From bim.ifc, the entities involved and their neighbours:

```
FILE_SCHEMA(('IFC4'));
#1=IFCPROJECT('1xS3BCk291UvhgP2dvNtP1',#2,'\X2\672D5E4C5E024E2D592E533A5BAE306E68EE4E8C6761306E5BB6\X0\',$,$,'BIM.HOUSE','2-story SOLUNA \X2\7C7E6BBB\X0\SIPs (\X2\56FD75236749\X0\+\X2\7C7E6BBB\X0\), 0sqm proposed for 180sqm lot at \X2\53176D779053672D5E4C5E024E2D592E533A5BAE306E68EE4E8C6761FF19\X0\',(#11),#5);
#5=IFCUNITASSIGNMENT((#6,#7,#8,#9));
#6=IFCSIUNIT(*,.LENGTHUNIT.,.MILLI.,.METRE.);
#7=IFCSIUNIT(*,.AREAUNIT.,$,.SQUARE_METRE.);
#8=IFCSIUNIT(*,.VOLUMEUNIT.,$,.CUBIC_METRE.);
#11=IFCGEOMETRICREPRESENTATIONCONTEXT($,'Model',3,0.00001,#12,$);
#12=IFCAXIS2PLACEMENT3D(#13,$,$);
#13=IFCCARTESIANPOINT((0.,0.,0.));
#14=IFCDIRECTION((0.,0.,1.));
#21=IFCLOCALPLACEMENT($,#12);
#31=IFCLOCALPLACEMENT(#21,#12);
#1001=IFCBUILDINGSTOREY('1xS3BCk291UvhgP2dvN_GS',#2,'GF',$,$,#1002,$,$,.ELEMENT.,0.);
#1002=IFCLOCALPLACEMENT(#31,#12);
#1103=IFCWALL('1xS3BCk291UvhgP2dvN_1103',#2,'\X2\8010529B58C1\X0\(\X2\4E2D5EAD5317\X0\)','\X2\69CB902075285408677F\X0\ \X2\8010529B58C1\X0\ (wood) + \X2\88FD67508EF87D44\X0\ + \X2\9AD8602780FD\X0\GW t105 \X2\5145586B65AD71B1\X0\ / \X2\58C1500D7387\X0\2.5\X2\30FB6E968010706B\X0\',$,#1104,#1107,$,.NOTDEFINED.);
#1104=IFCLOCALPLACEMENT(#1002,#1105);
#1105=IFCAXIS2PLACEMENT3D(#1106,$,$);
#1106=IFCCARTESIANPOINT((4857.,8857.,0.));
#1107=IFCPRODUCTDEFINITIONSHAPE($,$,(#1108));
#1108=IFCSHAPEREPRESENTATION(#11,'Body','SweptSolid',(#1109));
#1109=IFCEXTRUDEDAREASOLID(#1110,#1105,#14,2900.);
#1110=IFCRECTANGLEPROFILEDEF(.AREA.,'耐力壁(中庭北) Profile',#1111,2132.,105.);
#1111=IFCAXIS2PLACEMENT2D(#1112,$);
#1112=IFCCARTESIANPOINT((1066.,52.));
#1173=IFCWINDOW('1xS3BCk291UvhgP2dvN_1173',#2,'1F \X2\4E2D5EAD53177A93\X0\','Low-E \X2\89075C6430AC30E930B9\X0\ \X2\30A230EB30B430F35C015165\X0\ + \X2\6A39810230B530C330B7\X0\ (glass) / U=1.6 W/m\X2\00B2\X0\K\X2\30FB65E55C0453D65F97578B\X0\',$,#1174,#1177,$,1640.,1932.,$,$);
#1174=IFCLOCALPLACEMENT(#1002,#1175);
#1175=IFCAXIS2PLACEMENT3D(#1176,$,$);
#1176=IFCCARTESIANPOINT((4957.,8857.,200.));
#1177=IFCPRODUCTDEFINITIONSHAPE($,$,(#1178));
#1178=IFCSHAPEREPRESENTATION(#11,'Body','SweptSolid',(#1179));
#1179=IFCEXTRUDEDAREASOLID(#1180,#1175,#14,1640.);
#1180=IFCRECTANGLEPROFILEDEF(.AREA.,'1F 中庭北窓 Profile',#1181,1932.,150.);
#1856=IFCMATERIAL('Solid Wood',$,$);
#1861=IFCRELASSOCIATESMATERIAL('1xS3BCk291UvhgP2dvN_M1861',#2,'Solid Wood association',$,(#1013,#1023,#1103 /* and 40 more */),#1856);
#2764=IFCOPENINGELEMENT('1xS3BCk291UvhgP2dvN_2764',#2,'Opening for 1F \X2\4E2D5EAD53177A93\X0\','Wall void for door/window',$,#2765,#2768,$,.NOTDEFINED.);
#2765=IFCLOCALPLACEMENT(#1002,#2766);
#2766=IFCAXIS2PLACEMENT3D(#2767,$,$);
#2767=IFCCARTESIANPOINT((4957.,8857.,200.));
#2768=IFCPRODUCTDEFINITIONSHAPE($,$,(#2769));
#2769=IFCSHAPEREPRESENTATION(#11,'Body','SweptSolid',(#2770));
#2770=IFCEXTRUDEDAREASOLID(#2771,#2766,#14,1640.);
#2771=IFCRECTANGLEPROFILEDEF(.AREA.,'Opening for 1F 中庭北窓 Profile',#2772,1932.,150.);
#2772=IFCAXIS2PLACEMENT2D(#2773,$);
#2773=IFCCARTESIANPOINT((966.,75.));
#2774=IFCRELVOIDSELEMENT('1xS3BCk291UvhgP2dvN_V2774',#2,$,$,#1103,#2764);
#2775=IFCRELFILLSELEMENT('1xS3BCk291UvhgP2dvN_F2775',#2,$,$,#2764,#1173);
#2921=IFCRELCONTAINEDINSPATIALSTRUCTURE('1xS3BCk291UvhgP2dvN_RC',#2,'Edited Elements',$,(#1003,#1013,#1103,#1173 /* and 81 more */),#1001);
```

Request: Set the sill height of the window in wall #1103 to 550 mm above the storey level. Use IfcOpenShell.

```python
import numpy as np
import ifcopenshell
import ifcopenshell.api.geometry
import ifcopenshell.geom
import ifcopenshell.util.element
import ifcopenshell.util.placement
import ifcopenshell.util.shape
import ifcopenshell.util.unit

model = ifcopenshell.open("bim.ifc")
unit_scale = ifcopenshell.util.unit.calculate_unit_scale(model)

window = model.by_id(1173)
opening = window.FillsVoids[0].RelatingOpeningElement
storey = ifcopenshell.util.element.get_container(window, ifc_class="IfcBuildingStorey")
level = ifcopenshell.util.placement.get_local_placement(storey.ObjectPlacement)[2, 3]

# The opening's origin need not be at the sill, so measure its lowest point.
shape = ifcopenshell.geom.create_shape(ifcopenshell.geom.settings(), opening)
bottom = ifcopenshell.util.shape.get_shape_bottom_elevation(shape, shape.geometry) / unit_scale
dz = level + 550.0 - bottom

shift = np.array([0.0, 0.0, dz])
# The window is not placed relative to its opening, so move both.
for product in (opening, window):
    matrix = ifcopenshell.util.placement.get_local_placement(product.ObjectPlacement)
    matrix[:3, 3] += shift
    ifcopenshell.api.geometry.edit_object_placement(model, product=product, matrix=matrix, is_si=False)

print(f"moved by {dz * unit_scale:+.3f} m")

model.write("bim_v2.ifc")
```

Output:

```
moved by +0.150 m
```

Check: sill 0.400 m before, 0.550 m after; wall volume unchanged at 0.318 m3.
